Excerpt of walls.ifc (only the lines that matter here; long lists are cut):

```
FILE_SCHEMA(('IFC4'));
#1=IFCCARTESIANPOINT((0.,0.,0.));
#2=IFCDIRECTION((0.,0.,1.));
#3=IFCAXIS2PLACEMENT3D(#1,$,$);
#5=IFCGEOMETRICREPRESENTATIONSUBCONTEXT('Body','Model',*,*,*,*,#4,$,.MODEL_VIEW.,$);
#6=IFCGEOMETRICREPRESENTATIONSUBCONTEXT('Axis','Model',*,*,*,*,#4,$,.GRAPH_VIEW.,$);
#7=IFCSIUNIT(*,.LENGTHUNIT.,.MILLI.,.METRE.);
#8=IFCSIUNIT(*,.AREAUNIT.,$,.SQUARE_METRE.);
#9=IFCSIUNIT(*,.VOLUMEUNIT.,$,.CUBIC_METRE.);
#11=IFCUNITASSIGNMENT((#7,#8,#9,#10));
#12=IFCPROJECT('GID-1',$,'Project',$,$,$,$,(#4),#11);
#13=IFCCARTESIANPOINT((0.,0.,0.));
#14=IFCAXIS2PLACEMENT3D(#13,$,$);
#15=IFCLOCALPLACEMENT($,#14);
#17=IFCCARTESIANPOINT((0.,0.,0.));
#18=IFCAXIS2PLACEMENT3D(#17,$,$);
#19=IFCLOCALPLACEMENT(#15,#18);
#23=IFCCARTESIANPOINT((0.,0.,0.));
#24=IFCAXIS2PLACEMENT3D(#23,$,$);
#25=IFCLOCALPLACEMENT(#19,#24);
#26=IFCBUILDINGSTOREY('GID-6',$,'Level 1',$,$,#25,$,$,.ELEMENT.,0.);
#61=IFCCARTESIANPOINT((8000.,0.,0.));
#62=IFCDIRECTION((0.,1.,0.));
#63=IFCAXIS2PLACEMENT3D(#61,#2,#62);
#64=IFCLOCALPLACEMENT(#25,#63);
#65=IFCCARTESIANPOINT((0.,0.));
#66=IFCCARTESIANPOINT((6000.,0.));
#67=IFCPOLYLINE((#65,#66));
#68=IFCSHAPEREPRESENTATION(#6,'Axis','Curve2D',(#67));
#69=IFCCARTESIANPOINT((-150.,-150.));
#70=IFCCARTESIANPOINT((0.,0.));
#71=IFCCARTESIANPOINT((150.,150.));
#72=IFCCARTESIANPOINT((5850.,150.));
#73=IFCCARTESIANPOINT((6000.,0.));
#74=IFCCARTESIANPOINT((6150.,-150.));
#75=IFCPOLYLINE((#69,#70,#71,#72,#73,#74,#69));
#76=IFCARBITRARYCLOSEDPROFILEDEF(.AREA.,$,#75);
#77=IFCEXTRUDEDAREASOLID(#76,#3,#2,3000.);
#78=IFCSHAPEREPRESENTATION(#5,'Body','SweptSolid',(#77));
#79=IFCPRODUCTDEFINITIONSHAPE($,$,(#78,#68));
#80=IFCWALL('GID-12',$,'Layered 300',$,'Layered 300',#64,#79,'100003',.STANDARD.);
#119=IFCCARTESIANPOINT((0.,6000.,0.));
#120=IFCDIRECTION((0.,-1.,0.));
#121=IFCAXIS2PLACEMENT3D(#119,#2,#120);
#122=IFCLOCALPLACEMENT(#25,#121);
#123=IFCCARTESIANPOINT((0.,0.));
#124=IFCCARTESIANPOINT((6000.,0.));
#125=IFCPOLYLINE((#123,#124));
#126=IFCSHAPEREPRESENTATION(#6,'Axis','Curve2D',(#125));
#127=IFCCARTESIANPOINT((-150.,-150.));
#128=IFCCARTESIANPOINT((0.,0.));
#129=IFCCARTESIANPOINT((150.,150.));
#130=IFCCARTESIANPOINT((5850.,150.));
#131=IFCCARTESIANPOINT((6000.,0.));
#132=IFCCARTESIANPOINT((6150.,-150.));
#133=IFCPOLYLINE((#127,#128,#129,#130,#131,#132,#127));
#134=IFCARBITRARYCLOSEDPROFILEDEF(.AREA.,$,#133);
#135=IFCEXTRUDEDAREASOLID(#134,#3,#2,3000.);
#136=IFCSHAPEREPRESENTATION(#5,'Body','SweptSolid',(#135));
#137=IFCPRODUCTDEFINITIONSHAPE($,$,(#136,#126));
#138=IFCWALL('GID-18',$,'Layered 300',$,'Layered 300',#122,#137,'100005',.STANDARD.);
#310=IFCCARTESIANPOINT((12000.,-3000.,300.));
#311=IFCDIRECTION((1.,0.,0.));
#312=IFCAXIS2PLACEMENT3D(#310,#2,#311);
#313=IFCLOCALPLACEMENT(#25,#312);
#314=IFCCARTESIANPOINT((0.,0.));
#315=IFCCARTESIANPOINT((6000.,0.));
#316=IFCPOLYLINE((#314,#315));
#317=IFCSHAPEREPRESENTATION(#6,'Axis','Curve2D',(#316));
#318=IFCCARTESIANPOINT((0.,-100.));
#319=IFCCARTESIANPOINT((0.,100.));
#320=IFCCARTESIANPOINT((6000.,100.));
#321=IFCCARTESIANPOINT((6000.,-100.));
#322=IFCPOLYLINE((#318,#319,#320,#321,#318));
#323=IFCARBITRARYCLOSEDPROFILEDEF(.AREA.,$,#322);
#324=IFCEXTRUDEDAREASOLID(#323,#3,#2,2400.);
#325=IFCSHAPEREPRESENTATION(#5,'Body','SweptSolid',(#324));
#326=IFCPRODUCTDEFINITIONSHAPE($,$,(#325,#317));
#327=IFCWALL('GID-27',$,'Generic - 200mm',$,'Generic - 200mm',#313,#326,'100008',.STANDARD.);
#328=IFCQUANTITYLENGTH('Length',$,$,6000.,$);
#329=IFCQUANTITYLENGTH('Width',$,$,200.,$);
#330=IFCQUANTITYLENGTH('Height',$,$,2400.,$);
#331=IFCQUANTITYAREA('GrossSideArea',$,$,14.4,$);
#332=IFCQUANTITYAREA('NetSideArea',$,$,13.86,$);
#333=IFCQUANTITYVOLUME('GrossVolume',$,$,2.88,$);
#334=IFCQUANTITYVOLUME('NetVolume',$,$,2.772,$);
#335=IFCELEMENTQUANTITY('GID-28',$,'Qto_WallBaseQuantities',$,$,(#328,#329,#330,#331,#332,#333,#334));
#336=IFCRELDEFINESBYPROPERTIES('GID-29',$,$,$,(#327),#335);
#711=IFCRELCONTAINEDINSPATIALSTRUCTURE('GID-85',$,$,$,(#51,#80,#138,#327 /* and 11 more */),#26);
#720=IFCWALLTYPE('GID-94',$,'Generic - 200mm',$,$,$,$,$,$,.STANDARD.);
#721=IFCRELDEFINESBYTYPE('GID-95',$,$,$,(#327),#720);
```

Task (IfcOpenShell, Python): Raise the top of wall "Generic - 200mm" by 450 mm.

```python
import ifcopenshell
import ifcopenshell.api.pset
import ifcopenshell.geom
import ifcopenshell.util.element
import ifcopenshell.util.representation
import ifcopenshell.util.shape
import ifcopenshell.util.unit

model = ifcopenshell.open("walls.ifc")
unit_scale = ifcopenshell.util.unit.calculate_unit_scale(model)
area_scale = ifcopenshell.util.unit.calculate_unit_scale(model, "AREAUNIT")
volume_scale = ifcopenshell.util.unit.calculate_unit_scale(model, "VOLUMEUNIT")
settings = ifcopenshell.geom.settings()


def volume(element):
    """Net volume in cubic metres, openings subtracted."""
    shape = ifcopenshell.geom.create_shape(settings, element)
    return ifcopenshell.util.shape.get_volume(shape.geometry)


wall = model.by_guid("GID-27")
before = volume(wall)

body = ifcopenshell.util.representation.get_representation(wall, "Model", "Body")
solid = body.Items[0]
old_height = solid.Depth
solid.Depth += 0.45 / unit_scale
after = volume(wall)
thickness = 0.2  # wall thickness in metres

# Update the stored height, areas and volumes.
qto = model.by_id(ifcopenshell.util.element.get_pset(wall, "Qto_WallBaseQuantities", should_inherit=False)["id"])
ifcopenshell.api.pset.edit_qto(model, qto=qto, properties={
    "Height": solid.Depth,
    "GrossSideArea": ifcopenshell.util.element.get_pset(wall, "Qto_WallBaseQuantities", "GrossSideArea") * solid.Depth / old_height,
    "NetSideArea": after / thickness / area_scale,
    "GrossVolume": ifcopenshell.util.element.get_pset(wall, "Qto_WallBaseQuantities", "GrossVolume") * solid.Depth / old_height,
    "NetVolume": after / volume_scale,
})

print(f"height {old_height:g} -> {solid.Depth:g}, volume {before:.3f} -> {after:.3f} m3")

model.write("walls_rev.ifc")
```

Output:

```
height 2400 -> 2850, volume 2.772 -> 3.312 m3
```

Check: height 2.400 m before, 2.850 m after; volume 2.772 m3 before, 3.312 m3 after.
